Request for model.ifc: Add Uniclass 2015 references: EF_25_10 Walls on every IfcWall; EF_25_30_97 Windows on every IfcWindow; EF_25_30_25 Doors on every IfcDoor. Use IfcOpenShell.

First a look at what the model holds.

```python
import ifcopenshell

model = ifcopenshell.open("model.ifc")
print(model.schema)
print("classifications:", [c.Name for c in model.by_type("IfcClassification")])
for ifc_class in ("IfcDoor", "IfcRoof", "IfcStair", "IfcWall", "IfcWindow"):
    print(ifc_class, len(model.by_type(ifc_class)))
```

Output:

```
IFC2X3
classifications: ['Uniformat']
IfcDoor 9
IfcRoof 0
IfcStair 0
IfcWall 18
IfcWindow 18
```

```python
import ifcopenshell
import ifcopenshell.api.classification

model = ifcopenshell.open("model.ifc")

# IFC2X3 requires Source and Edition and has no link from the project to the system.
system = model.create_entity("IfcClassification", Source="NBS", Edition="2015", Name="Uniclass 2015")

codes = {
    "IfcWall": ("EF_25_10", "Walls"),
    "IfcWindow": ("EF_25_30_97", "Windows"),
    "IfcDoor": ("EF_25_30_25", "Doors"),
}
for ifc_class, (code, name) in codes.items():
    products = model.by_type(ifc_class)
    ifcopenshell.api.classification.add_reference(
        model, products=products, classification=system, identification=code, name=name
    )
    print(code, len(products))

model.write("model_edited.ifc")
```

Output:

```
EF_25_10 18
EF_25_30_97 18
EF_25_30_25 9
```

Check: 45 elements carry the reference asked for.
